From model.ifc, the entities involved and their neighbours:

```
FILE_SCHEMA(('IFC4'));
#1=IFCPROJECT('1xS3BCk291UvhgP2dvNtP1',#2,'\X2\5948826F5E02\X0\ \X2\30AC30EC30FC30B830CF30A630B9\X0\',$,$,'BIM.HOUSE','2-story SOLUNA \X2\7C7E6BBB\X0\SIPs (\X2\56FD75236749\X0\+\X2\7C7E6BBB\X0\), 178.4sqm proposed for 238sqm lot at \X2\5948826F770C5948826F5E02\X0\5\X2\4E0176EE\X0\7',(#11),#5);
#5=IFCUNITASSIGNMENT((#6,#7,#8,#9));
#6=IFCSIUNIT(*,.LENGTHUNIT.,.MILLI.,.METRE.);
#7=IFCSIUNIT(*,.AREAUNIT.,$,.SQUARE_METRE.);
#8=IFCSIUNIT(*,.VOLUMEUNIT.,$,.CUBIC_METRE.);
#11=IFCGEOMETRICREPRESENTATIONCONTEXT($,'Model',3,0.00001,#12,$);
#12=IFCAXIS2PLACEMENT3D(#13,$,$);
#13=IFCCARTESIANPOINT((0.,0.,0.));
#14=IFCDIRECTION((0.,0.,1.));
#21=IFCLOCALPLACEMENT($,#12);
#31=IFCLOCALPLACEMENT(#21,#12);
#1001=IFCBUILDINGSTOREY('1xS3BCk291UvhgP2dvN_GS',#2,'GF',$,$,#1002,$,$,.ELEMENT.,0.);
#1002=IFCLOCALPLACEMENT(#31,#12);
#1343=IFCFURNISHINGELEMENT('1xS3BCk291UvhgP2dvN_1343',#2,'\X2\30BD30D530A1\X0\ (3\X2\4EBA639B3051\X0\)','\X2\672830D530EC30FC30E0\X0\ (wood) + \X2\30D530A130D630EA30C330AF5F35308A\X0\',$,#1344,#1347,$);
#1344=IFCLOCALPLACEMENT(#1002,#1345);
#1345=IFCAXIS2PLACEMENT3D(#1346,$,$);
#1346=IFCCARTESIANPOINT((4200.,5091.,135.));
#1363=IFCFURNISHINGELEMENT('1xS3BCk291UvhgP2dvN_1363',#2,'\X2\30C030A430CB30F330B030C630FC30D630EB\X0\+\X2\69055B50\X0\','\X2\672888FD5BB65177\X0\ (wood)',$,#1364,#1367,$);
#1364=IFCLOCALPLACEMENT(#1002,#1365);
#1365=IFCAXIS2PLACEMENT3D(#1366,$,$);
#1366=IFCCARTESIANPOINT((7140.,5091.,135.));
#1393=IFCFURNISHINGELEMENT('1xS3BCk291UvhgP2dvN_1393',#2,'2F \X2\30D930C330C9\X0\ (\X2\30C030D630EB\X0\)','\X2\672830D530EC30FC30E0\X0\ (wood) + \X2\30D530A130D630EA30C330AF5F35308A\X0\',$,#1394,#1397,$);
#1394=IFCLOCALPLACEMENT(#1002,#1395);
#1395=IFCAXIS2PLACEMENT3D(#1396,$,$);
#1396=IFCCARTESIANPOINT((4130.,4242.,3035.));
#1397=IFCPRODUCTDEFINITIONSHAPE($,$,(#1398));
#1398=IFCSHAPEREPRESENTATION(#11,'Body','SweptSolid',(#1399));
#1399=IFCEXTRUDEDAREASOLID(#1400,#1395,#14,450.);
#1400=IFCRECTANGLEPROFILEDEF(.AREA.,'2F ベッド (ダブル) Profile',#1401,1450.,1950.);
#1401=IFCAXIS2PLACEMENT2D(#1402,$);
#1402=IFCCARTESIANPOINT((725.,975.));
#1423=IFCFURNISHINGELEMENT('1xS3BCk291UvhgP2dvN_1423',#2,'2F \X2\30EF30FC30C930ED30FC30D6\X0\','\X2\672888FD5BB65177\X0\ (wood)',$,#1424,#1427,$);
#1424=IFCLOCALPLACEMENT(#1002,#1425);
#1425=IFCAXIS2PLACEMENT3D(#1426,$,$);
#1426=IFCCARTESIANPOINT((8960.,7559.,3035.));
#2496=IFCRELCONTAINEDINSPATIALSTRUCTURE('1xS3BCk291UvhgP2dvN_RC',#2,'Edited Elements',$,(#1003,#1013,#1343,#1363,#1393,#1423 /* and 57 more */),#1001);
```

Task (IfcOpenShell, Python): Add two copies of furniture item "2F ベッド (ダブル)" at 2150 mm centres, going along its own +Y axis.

```python
import ifcopenshell
import ifcopenshell.api.geometry
import ifcopenshell.api.root
import ifcopenshell.util.element
import ifcopenshell.util.placement

model = ifcopenshell.open("model.ifc")


def reuse_history(source, copy):
    """copy_class also copies each property set's owner history, people and application; keep the originals."""
    for rel in copy.IsDefinedBy:
        if rel.is_a("IfcRelDefinesByProperties") and (history := rel.RelatingPropertyDefinition.OwnerHistory):
            rel.RelatingPropertyDefinition.OwnerHistory = source.OwnerHistory
            ifcopenshell.util.element.remove_deep2(model, history)


source = model.by_guid("1xS3BCk291UvhgP2dvN_1393")
base = ifcopenshell.util.placement.get_local_placement(source.ObjectPlacement)
step = base[:3, 1] * 2150.0

for i in range(1, 3):
    copy = ifcopenshell.api.root.copy_class(model, product=source)
    copy.Representation = ifcopenshell.util.element.copy_deep(
        model, source.Representation, exclude=["IfcGeometricRepresentationContext", "IfcRepresentationMap"]
    )
    reuse_history(source, copy)
    matrix = base.copy()
    matrix[:3, 3] += i * step
    print("added at", matrix[:3, 3].round(3) + 0.0)
    ifcopenshell.api.geometry.edit_object_placement(model, product=copy, matrix=matrix, is_si=False)

model.write("model_rev.ifc")
```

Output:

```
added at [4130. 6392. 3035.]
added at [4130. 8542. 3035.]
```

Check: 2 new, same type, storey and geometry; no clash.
